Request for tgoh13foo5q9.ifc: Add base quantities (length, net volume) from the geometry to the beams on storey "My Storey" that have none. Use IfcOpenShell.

First a look at what the model holds.

```python
import ifcopenshell
import ifcopenshell.util.element
import ifcopenshell.util.unit

model = ifcopenshell.open("tgoh13foo5q9.ifc")
print(model.schema)
for unit_type in ("LENGTHUNIT", "AREAUNIT", "VOLUMEUNIT"):
    print(unit_type, ifcopenshell.util.unit.calculate_unit_scale(model, unit_type))
storey = next(s for s in model.by_type("IfcBuildingStorey") if s.Name == "My Storey")
beams = [e for e in ifcopenshell.util.element.get_decomposition(storey) if e.is_a("IfcBeam")]
for e in sorted(beams, key=lambda e: e.id()):
    print(e.id(), e.is_a(), e.Name, list(ifcopenshell.util.element.get_psets(e, qtos_only=True)), sep=" | ")
```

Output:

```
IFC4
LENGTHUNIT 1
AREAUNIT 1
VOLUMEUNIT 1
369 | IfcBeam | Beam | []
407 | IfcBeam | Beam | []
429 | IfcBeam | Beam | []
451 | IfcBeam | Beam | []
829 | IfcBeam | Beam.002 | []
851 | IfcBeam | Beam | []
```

```python
import ifcopenshell
import ifcopenshell.api.pset
import ifcopenshell.geom
import ifcopenshell.util.element
import ifcopenshell.util.shape
import ifcopenshell.util.unit

model = ifcopenshell.open("tgoh13foo5q9.ifc")
unit_scale = ifcopenshell.util.unit.calculate_unit_scale(model)
volume_scale = ifcopenshell.util.unit.calculate_unit_scale(model, "VOLUMEUNIT")
settings = ifcopenshell.geom.settings()

storey = next(s for s in model.by_type("IfcBuildingStorey") if s.Name == "My Storey")
beams = [e for e in ifcopenshell.util.element.get_decomposition(storey) if e.is_a("IfcBeam")]

for e in sorted(beams, key=lambda e: e.id()):
    if ifcopenshell.util.element.get_psets(e, qtos_only=True, should_inherit=False):
        continue
    # Geometry comes back in metres, in the element's own axes.
    shape = ifcopenshell.geom.create_shape(settings, e)
    values = {
        "Length": ifcopenshell.util.shape.get_max_xyz(shape.geometry) / unit_scale,
        "NetVolume": ifcopenshell.util.shape.get_volume(shape.geometry) / volume_scale,
    }
    qto = ifcopenshell.api.pset.add_qto(model, product=e, name="Qto_BeamBaseQuantities")
    ifcopenshell.api.pset.edit_qto(model, qto=qto, properties=values)
    print(e.id(), {k: round(v, 3) for k, v in values.items()})

model.write("tgoh13foo5q9_rev.ifc")
```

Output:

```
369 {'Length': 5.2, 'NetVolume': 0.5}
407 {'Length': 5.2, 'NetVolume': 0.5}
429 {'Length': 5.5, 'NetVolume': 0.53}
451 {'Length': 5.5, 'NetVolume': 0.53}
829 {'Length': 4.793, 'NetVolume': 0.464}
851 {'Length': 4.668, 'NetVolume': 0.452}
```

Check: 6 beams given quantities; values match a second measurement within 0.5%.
